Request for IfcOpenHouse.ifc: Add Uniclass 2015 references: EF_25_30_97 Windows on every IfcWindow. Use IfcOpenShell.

First a look at what the model holds.

```python
import ifcopenshell

model = ifcopenshell.open("IfcOpenHouse.ifc")
print(model.schema)
print("classifications:", [c.Name for c in model.by_type("IfcClassification")])
for ifc_class in ("IfcDoor", "IfcRoof", "IfcStair", "IfcWall", "IfcWindow"):
    print(ifc_class, len(model.by_type(ifc_class)))
```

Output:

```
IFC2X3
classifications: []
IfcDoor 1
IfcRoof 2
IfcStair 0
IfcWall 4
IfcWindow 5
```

```python
import ifcopenshell
import ifcopenshell.api.classification

model = ifcopenshell.open("IfcOpenHouse.ifc")

# IFC2X3 requires Source and Edition and has no link from the project to the system.
system = model.create_entity("IfcClassification", Source="NBS", Edition="2015", Name="Uniclass 2015")

codes = {
    "IfcWindow": ("EF_25_30_97", "Windows"),
}
for ifc_class, (code, name) in codes.items():
    products = model.by_type(ifc_class)
    ifcopenshell.api.classification.add_reference(
        model, products=products, classification=system, identification=code, name=name
    )
    print(code, len(products))

model.write("IfcOpenHouse_rev.ifc")
```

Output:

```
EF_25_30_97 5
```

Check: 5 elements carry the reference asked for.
